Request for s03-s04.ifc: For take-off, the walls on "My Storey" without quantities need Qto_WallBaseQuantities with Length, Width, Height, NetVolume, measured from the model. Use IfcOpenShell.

First a look at what the model holds.

```python
import ifcopenshell
import ifcopenshell.util.element
import ifcopenshell.util.unit

model = ifcopenshell.open("s03-s04.ifc")
print(model.schema)
for unit_type in ("LENGTHUNIT", "AREAUNIT", "VOLUMEUNIT"):
    print(unit_type, ifcopenshell.util.unit.calculate_unit_scale(model, unit_type))
storey = next(s for s in model.by_type("IfcBuildingStorey") if s.Name == "My Storey")
walls = [e for e in ifcopenshell.util.element.get_decomposition(storey) if e.is_a("IfcWall")]
for e in sorted(walls, key=lambda e: e.id()):
    print(e.id(), e.is_a(), e.Name, list(ifcopenshell.util.element.get_psets(e, qtos_only=True)), sep=" | ")
```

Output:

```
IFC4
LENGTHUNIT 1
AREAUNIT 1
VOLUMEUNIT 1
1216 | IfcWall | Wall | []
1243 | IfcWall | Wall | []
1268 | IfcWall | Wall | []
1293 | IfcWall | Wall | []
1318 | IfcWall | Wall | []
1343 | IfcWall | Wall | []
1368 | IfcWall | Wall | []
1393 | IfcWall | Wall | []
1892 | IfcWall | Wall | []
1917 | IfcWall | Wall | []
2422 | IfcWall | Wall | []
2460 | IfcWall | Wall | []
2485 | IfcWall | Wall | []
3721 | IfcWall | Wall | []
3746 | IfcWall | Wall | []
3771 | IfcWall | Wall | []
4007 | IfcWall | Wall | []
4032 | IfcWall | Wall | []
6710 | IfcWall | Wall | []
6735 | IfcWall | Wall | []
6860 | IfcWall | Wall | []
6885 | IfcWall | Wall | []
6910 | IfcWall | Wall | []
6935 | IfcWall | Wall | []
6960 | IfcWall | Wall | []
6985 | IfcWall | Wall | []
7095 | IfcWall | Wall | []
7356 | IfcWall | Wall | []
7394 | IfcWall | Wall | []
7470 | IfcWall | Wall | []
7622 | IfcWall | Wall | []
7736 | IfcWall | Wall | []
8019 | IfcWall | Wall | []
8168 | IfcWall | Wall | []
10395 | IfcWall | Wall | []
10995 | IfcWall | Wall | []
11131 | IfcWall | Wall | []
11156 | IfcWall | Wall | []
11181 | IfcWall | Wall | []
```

```python
import ifcopenshell
import ifcopenshell.api.pset
import ifcopenshell.geom
import ifcopenshell.util.element
import ifcopenshell.util.shape
import ifcopenshell.util.unit

model = ifcopenshell.open("s03-s04.ifc")
unit_scale = ifcopenshell.util.unit.calculate_unit_scale(model)
volume_scale = ifcopenshell.util.unit.calculate_unit_scale(model, "VOLUMEUNIT")
settings = ifcopenshell.geom.settings()

storey = next(s for s in model.by_type("IfcBuildingStorey") if s.Name == "My Storey")
walls = [e for e in ifcopenshell.util.element.get_decomposition(storey) if e.is_a("IfcWall")]

for e in sorted(walls, key=lambda e: e.id()):
    if ifcopenshell.util.element.get_psets(e, qtos_only=True, should_inherit=False):
        continue
    # Geometry comes back in metres, in the element's own axes.
    shape = ifcopenshell.geom.create_shape(settings, e)
    values = {
        "Length": ifcopenshell.util.shape.get_x(shape.geometry) / unit_scale,
        "Width": ifcopenshell.util.shape.get_y(shape.geometry) / unit_scale,
        "Height": ifcopenshell.util.shape.get_z(shape.geometry) / unit_scale,
        "NetVolume": ifcopenshell.util.shape.get_volume(shape.geometry) / volume_scale,
    }
    qto = ifcopenshell.api.pset.add_qto(model, product=e, name="Qto_WallBaseQuantities")
    ifcopenshell.api.pset.edit_qto(model, qto=qto, properties=values)
    print(e.id(), {k: round(v, 3) for k, v in values.items()})

model.write("s03-s04_updated.ifc")
```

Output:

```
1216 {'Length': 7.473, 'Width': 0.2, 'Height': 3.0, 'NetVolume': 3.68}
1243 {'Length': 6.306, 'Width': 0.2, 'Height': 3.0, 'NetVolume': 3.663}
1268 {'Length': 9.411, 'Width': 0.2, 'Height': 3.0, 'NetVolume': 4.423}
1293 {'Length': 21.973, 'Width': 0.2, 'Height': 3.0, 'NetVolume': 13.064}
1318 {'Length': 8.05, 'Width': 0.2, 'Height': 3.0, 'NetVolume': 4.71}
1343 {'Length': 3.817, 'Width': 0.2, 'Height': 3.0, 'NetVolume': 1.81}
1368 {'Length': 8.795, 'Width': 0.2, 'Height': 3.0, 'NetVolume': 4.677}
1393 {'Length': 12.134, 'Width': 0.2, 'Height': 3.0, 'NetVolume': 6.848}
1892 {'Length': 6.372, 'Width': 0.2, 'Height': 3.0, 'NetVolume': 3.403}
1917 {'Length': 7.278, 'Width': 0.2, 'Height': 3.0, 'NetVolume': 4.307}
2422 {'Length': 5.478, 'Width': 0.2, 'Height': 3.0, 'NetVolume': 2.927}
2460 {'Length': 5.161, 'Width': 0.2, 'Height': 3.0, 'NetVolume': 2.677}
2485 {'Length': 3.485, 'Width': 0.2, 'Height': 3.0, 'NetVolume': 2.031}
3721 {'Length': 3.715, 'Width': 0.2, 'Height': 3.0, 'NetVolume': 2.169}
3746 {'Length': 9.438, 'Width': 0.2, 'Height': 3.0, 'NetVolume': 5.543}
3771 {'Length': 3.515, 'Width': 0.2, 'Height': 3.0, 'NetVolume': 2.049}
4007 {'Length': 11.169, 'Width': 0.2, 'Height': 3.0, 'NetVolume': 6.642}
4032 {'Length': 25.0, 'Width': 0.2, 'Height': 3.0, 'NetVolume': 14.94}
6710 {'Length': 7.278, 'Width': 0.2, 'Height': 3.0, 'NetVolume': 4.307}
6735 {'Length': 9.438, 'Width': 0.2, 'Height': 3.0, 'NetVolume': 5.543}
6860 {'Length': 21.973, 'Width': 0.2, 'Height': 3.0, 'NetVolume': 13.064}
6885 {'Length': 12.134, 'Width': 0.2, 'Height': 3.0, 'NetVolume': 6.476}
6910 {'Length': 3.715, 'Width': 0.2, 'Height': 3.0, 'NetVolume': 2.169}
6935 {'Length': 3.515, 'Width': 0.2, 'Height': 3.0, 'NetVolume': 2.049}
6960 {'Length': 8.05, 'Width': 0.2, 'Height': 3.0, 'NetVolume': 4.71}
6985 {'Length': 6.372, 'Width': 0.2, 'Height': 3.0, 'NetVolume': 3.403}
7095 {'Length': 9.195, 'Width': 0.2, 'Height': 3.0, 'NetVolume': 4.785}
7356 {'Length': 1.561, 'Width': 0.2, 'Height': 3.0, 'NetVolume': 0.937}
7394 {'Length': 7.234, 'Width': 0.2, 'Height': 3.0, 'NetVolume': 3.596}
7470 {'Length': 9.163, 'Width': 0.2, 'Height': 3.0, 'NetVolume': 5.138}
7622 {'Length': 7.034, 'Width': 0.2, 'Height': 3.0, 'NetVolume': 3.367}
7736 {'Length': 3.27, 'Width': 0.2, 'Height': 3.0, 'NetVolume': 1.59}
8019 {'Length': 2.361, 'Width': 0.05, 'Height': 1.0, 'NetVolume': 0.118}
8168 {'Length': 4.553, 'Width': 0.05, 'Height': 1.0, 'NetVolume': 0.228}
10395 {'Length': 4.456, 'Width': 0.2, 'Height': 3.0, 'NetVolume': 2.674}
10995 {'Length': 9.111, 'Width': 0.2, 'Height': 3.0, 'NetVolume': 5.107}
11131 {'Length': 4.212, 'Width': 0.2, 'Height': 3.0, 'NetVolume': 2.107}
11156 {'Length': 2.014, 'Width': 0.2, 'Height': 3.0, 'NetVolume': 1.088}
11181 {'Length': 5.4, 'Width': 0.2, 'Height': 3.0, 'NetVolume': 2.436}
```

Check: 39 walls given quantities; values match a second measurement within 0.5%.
